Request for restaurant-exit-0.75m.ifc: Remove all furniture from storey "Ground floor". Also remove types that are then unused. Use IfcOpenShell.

First a look at what the model holds.

```python
import ifcopenshell
import ifcopenshell.util.element

model = ifcopenshell.open("restaurant-exit-0.75m.ifc")
print(model.schema)
storey = next(s for s in model.by_type("IfcBuildingStorey") if s.Name == "Ground floor")
furniture = [e for e in ifcopenshell.util.element.get_decomposition(storey) if e.is_a("IfcFurnishingElement")]
seen = {}
for e in furniture:
    element_type = ifcopenshell.util.element.get_type(e)
    name = element_type.Name if element_type not in (None, e) else None
    seen[name] = seen.get(name, 0) + 1
for name, count in sorted(seen.items(), key=str):
    print(count, "x", name)
```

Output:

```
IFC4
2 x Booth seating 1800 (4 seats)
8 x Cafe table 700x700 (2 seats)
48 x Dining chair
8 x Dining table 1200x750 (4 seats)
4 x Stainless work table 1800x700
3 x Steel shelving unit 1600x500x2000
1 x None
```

```python
import ifcopenshell
import ifcopenshell.api.root
import ifcopenshell.util.element

model = ifcopenshell.open("restaurant-exit-0.75m.ifc")

storey = next(s for s in model.by_type("IfcBuildingStorey") if s.Name == "Ground floor")
furniture = [e for e in ifcopenshell.util.element.get_decomposition(storey) if e.is_a("IfcFurnishingElement")]
types = {ifcopenshell.util.element.get_type(e) for e in furniture} - {None, *furniture}

for e in furniture:
    ifcopenshell.api.root.remove_product(model, product=e)
print(len(furniture), "removed")

unused = [t for t in types if not ifcopenshell.util.element.get_types(t)]
for t in unused:
    ifcopenshell.api.root.remove_product(model, product=t)
print(len(unused), "unused types removed")

model.write("restaurant-exit-0.75m_v2.ifc")
```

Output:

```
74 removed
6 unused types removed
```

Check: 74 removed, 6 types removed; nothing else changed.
